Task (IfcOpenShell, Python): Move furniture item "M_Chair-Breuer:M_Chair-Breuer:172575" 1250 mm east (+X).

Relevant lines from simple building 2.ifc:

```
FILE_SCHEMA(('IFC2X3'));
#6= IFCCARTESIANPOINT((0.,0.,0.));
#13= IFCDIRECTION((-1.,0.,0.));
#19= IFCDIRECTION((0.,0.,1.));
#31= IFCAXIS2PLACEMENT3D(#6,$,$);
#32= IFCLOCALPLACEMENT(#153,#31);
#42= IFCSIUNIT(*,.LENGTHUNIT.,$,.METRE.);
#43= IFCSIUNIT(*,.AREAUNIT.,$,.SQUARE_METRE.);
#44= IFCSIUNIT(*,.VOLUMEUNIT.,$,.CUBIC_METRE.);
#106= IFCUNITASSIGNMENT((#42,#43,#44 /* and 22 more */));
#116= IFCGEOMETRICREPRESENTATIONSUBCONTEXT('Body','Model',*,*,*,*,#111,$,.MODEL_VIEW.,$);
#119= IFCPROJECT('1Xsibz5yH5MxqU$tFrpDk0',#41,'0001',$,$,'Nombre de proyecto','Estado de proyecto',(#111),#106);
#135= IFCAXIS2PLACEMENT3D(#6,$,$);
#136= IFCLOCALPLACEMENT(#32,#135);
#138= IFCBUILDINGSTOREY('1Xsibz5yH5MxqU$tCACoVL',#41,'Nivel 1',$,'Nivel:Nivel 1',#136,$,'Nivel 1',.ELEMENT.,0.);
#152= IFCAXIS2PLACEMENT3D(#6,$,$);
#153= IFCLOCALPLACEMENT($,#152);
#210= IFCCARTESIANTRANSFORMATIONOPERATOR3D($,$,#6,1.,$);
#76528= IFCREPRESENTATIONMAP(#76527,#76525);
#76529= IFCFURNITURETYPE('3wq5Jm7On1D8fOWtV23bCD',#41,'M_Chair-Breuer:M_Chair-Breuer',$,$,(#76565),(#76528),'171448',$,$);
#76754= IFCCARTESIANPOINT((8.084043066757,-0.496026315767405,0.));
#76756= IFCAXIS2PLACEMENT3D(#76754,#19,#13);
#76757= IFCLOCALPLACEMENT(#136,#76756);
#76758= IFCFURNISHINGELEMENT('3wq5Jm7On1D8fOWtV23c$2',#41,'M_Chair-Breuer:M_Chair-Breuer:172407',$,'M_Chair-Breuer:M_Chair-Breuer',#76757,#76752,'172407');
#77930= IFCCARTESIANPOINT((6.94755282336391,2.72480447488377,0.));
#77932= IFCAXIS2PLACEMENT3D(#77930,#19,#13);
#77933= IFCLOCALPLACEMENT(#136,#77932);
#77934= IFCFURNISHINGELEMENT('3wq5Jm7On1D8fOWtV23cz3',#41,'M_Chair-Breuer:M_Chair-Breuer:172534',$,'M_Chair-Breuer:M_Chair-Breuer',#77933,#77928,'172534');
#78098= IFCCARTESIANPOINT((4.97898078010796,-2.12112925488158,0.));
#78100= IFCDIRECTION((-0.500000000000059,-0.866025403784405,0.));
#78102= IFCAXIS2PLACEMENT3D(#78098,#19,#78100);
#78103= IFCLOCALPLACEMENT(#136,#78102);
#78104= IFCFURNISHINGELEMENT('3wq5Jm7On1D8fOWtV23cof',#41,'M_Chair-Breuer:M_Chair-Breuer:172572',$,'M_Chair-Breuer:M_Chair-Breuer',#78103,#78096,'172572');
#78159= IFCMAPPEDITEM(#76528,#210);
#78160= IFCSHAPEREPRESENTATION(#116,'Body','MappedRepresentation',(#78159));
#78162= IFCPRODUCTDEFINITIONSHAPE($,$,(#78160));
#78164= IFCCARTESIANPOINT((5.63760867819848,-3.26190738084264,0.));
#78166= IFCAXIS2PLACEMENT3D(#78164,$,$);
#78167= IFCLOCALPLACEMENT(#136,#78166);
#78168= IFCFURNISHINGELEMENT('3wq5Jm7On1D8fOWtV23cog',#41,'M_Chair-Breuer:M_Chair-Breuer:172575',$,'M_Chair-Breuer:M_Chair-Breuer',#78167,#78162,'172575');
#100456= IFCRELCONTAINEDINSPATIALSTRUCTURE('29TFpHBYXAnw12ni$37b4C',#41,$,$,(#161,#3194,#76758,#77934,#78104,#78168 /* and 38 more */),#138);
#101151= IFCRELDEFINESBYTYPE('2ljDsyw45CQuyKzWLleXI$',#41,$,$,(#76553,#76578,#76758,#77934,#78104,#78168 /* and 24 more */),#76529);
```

```python
import ifcopenshell
import ifcopenshell.api.geometry
import ifcopenshell.util.placement
import ifcopenshell.util.unit

model = ifcopenshell.open("simple building 2.ifc")
unit_scale = ifcopenshell.util.unit.calculate_unit_scale(model)

item = model.by_guid("3wq5Jm7On1D8fOWtV23cog")
matrix = ifcopenshell.util.placement.get_local_placement(item.ObjectPlacement)
matrix[0, 3] += 1.25 / unit_scale
ifcopenshell.api.geometry.edit_object_placement(model, product=item, matrix=matrix, is_si=False)

print(ifcopenshell.util.placement.get_local_placement(item.ObjectPlacement).round(3) + 0.0)

model.write("simple building 2_rev.ifc")
```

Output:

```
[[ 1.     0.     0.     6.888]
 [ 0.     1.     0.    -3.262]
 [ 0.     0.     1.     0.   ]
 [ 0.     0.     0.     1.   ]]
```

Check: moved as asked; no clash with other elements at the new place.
